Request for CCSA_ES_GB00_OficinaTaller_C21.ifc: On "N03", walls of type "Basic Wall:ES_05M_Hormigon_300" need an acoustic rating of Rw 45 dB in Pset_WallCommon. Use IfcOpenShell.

First a look at what the model holds.

```python
import ifcopenshell
import ifcopenshell.util.element

model = ifcopenshell.open("CCSA_ES_GB00_OficinaTaller_C21.ifc")
print(model.schema)
storey = next(s for s in model.by_type("IfcBuildingStorey") if s.Name == "N03")
walls = [e for e in ifcopenshell.util.element.get_decomposition(storey) if e.is_a("IfcWall")]
seen = {}
for e in walls:
    element_type = ifcopenshell.util.element.get_type(e)
    key = (element_type.Name if element_type != e and element_type else None, ifcopenshell.util.element.get_pset(e, "Pset_WallCommon", "AcousticRating"))
    seen[key] = seen.get(key, 0) + 1
for (name, value), count in sorted(seen.items(), key=str):
    print(count, "x", name, "|", value)
```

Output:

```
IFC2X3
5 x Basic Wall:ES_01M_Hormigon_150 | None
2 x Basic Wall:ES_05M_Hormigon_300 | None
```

```python
import ifcopenshell
import ifcopenshell.api.pset
import ifcopenshell.util.element

model = ifcopenshell.open("CCSA_ES_GB00_OficinaTaller_C21.ifc")

storey = next(s for s in model.by_type("IfcBuildingStorey") if s.Name == "N03")
walls = [e for e in ifcopenshell.util.element.get_decomposition(storey) if e.is_a("IfcWall")]

count = 0
for e in walls:
    element_type = ifcopenshell.util.element.get_type(e)
    if element_type in (None, e) or element_type.Name != "Basic Wall:ES_05M_Hormigon_300":
        continue
    # add_pset returns the element's existing set when there is one.
    pset = ifcopenshell.api.pset.add_pset(model, product=e, name="Pset_WallCommon")
    ifcopenshell.api.pset.edit_pset(model, pset=pset, properties={"AcousticRating": "Rw 45 dB"})
    count += 1

print(count, "walls updated")

model.write("CCSA_ES_GB00_OficinaTaller_C21_edited.ifc")
```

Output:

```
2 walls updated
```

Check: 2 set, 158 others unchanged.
